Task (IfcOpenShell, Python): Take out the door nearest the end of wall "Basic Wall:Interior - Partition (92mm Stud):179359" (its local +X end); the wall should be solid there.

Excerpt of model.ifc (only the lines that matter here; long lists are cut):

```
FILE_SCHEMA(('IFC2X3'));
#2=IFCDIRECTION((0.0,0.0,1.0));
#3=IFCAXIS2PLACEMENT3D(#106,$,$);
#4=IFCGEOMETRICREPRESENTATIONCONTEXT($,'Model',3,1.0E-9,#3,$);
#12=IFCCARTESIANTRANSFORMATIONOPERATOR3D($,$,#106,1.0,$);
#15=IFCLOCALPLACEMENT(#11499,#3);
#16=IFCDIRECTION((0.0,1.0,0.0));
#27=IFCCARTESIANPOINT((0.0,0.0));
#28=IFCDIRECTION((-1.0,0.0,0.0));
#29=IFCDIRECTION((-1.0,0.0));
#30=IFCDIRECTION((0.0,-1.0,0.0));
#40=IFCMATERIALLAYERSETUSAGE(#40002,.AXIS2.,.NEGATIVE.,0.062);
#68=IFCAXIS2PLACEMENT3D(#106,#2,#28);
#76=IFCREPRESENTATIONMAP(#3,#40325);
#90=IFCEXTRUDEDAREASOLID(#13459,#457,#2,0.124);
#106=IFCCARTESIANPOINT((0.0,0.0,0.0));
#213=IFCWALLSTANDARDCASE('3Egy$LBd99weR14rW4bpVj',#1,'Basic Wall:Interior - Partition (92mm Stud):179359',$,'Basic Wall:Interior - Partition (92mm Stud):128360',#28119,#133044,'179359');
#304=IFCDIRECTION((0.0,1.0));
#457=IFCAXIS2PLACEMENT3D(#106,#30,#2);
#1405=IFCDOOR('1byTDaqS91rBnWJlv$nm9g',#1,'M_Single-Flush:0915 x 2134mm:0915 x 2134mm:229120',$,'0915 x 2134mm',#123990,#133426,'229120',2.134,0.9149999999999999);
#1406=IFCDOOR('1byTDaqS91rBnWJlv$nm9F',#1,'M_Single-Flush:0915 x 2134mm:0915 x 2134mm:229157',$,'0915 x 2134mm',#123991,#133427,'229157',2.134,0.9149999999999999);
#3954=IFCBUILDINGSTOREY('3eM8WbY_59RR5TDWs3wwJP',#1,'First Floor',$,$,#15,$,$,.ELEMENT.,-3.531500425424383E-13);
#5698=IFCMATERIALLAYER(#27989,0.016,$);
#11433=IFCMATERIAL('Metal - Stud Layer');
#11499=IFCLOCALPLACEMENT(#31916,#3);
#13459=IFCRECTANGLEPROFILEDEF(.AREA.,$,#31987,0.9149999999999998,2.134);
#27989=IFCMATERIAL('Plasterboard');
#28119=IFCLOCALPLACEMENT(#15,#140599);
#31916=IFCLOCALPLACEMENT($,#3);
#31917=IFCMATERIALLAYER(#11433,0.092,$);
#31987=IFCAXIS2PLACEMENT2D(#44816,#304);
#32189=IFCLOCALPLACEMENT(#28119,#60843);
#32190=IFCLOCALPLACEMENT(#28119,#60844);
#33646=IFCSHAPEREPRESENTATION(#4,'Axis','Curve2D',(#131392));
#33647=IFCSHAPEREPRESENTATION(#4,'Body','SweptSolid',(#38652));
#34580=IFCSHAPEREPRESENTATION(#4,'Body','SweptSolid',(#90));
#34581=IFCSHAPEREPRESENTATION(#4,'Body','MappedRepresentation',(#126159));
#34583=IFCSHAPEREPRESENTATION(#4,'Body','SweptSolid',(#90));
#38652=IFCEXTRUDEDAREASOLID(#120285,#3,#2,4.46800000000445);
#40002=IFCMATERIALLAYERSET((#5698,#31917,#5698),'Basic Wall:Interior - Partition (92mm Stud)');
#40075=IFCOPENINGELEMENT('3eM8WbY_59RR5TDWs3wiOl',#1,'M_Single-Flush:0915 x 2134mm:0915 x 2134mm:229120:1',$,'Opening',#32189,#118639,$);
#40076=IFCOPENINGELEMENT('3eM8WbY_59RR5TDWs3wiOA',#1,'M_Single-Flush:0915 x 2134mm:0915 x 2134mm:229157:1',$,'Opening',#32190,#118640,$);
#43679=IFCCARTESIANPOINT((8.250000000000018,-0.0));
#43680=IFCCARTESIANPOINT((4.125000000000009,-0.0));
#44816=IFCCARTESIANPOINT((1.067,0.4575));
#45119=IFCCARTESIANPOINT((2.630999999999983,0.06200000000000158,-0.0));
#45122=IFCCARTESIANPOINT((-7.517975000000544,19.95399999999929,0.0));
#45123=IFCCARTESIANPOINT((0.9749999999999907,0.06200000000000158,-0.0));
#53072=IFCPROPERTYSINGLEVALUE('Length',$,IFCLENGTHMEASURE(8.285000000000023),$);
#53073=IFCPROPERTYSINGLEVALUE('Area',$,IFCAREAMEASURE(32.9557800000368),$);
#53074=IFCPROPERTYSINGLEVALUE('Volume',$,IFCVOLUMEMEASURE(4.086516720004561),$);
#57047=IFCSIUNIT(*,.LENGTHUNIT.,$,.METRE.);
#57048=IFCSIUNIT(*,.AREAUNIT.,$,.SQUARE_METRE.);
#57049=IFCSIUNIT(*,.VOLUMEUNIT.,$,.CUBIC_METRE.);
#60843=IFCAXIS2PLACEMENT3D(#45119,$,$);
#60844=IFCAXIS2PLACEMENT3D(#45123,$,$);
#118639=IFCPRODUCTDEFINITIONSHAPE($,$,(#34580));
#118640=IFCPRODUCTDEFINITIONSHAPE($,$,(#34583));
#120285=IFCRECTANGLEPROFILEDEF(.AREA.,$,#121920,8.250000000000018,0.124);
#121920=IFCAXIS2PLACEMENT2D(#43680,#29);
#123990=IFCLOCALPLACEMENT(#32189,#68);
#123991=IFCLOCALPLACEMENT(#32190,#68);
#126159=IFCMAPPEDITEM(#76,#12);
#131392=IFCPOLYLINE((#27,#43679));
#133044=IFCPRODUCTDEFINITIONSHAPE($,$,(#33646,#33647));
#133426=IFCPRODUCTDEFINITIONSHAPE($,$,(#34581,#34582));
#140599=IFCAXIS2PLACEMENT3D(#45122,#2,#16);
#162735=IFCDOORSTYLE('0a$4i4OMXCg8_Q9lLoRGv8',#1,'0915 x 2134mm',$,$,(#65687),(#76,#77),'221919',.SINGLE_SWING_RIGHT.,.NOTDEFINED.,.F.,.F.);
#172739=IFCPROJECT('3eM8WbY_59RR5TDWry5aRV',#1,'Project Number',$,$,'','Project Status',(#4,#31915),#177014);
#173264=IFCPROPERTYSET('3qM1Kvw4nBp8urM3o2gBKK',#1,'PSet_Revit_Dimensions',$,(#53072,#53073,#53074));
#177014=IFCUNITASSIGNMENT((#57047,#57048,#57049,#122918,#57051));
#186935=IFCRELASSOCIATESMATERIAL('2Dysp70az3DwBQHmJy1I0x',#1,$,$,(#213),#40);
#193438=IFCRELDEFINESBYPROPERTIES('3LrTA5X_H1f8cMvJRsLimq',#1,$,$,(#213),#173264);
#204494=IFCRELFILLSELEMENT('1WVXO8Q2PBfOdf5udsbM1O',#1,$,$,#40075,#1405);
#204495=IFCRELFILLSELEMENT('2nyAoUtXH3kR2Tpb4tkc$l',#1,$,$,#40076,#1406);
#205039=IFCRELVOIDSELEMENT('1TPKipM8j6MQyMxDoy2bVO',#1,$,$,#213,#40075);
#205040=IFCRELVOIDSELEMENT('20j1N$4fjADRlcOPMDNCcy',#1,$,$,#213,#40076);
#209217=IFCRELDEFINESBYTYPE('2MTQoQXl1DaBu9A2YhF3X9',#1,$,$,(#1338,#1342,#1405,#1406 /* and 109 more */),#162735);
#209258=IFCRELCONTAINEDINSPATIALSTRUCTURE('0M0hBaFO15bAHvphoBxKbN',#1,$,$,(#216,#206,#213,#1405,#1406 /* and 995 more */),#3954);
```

```python
import ifcopenshell
import ifcopenshell.api.feature
import ifcopenshell.api.pset
import ifcopenshell.api.root
import ifcopenshell.geom
import ifcopenshell.util.element
import ifcopenshell.util.shape
import ifcopenshell.util.unit

model = ifcopenshell.open("model.ifc")
area_scale = ifcopenshell.util.unit.calculate_unit_scale(model, "AREAUNIT")
volume_scale = ifcopenshell.util.unit.calculate_unit_scale(model, "VOLUMEUNIT")
settings = ifcopenshell.geom.settings()


def volume(element):
    """Net volume in cubic metres, openings subtracted."""
    shape = ifcopenshell.geom.create_shape(settings, element)
    return ifcopenshell.util.shape.get_volume(shape.geometry)


door = model.by_guid("1byTDaqS91rBnWJlv$nm9g")
opening = door.FillsVoids[0].RelatingOpeningElement
wall = opening.VoidsElements[0].RelatingBuildingElement
before = volume(wall)

ifcopenshell.api.root.remove_product(model, product=door)
ifcopenshell.api.feature.remove_feature(model, feature=opening)

after = volume(wall)
thickness = 0.124  # wall thickness in metres

# Update the wall's stored quantities.
pset = model.by_id(ifcopenshell.util.element.get_pset(wall, "PSet_Revit_Dimensions", should_inherit=False)["id"])
ifcopenshell.api.pset.edit_pset(model, pset=pset, properties={
    "Area": model.create_entity("IfcAreaMeasure", after / thickness / area_scale),
    "Volume": model.create_entity("IfcVolumeMeasure", after / volume_scale),
})

print(f"wall volume {before:.3f} -> {after:.3f} m3")

model.write("model_rev.ifc")
```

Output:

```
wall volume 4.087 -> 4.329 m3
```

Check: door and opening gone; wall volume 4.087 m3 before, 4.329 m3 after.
